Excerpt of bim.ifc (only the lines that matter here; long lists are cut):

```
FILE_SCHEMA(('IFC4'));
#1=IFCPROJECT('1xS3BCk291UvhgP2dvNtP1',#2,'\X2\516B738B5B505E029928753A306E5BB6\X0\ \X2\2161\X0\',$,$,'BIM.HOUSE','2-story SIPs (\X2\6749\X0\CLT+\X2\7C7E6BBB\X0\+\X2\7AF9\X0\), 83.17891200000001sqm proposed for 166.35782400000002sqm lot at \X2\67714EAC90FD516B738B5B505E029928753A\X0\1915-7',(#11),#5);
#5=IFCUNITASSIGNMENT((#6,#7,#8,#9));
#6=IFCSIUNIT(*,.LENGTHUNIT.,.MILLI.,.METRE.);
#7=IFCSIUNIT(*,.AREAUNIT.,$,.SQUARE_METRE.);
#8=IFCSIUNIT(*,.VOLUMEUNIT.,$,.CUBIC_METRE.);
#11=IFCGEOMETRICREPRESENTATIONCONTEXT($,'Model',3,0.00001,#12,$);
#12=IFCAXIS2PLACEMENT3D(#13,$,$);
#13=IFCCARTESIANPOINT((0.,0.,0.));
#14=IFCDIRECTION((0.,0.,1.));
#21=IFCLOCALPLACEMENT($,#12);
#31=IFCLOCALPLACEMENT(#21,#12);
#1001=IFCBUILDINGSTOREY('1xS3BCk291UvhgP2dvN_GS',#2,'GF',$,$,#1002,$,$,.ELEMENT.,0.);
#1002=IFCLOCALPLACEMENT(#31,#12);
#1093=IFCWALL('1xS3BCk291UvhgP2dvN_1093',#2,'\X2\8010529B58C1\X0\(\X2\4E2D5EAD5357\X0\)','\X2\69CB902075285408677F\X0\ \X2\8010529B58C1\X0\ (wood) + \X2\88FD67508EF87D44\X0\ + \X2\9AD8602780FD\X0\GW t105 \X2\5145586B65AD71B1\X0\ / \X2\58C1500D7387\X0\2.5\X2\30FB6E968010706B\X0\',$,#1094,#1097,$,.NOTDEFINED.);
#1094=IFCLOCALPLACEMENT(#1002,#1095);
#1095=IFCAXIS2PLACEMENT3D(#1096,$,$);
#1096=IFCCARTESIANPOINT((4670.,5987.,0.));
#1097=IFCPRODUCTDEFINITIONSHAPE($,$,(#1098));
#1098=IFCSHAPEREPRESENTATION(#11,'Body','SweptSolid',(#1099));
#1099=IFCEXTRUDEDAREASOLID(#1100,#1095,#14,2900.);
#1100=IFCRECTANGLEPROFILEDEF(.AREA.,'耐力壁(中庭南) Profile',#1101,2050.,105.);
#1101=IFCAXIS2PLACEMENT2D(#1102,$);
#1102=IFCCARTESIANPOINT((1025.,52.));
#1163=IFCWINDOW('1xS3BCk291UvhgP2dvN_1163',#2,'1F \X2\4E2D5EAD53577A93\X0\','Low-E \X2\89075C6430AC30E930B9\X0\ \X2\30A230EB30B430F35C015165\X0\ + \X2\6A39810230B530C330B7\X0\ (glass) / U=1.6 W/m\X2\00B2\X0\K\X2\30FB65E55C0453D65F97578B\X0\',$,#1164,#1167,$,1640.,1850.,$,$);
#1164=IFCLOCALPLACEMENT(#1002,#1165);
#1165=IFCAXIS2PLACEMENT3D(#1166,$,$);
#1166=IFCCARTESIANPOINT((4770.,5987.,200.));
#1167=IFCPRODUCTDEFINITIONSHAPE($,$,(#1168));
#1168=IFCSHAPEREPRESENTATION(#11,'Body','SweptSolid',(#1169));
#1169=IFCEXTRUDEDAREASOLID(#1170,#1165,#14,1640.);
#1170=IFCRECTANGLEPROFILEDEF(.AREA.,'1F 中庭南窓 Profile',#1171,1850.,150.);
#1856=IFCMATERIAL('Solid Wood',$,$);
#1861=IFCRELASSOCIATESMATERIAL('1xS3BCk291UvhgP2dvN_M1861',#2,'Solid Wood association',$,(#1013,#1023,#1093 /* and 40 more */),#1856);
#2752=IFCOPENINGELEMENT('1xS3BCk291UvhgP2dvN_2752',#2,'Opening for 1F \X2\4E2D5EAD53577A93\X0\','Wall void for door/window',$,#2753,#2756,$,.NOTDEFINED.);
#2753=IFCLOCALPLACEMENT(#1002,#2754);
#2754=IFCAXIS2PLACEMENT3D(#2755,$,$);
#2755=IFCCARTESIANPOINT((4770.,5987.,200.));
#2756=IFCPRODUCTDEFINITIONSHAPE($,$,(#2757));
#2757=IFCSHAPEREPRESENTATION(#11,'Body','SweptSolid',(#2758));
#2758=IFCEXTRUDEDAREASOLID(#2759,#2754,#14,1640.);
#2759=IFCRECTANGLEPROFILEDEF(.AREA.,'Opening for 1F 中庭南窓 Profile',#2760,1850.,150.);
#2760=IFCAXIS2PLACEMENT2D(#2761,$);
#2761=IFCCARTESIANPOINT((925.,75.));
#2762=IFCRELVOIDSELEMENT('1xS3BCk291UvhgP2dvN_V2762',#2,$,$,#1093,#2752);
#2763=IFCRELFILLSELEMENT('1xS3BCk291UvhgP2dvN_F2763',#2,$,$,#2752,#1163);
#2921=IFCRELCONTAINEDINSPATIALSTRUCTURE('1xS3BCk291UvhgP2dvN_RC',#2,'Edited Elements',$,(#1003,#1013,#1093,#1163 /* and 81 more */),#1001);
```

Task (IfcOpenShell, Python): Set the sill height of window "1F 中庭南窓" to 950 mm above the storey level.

```python
import numpy as np
import ifcopenshell
import ifcopenshell.api.geometry
import ifcopenshell.geom
import ifcopenshell.util.element
import ifcopenshell.util.placement
import ifcopenshell.util.shape
import ifcopenshell.util.unit

model = ifcopenshell.open("bim.ifc")
unit_scale = ifcopenshell.util.unit.calculate_unit_scale(model)

window = model.by_guid("1xS3BCk291UvhgP2dvN_1163")
opening = window.FillsVoids[0].RelatingOpeningElement
storey = ifcopenshell.util.element.get_container(window, ifc_class="IfcBuildingStorey")
level = ifcopenshell.util.placement.get_local_placement(storey.ObjectPlacement)[2, 3]

# The opening's origin need not be at the sill, so measure its lowest point.
shape = ifcopenshell.geom.create_shape(ifcopenshell.geom.settings(), opening)
bottom = ifcopenshell.util.shape.get_shape_bottom_elevation(shape, shape.geometry) / unit_scale
dz = level + 950.0 - bottom

shift = np.array([0.0, 0.0, dz])
# The window is not placed relative to its opening, so move both.
for product in (opening, window):
    matrix = ifcopenshell.util.placement.get_local_placement(product.ObjectPlacement)
    matrix[:3, 3] += shift
    ifcopenshell.api.geometry.edit_object_placement(model, product=product, matrix=matrix, is_si=False)

print(f"moved by {dz * unit_scale:+.3f} m")

model.write("bim-out.ifc")
```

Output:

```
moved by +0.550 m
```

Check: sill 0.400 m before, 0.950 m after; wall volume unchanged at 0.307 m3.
